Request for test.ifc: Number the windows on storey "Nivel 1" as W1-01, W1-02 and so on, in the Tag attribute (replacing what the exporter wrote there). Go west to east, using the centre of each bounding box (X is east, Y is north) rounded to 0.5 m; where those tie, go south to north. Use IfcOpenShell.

First a look at what the model holds.

```python
import ifcopenshell
import ifcopenshell.util.element
import ifcopenshell.util.placement

model = ifcopenshell.open("test.ifc")
print(model.schema)
storey = next(s for s in model.by_type("IfcBuildingStorey") if s.Name == "Nivel 1")
windows = [e for e in ifcopenshell.util.element.get_decomposition(storey) if e.is_a("IfcWindow")]
for e in sorted(windows, key=lambda e: e.id()):
    origin = ifcopenshell.util.placement.get_local_placement(e.ObjectPlacement)[:3, 3]
    print(e.id(), e.Tag, e.Name, origin.round(2) + 0.0, sep=" | ")
```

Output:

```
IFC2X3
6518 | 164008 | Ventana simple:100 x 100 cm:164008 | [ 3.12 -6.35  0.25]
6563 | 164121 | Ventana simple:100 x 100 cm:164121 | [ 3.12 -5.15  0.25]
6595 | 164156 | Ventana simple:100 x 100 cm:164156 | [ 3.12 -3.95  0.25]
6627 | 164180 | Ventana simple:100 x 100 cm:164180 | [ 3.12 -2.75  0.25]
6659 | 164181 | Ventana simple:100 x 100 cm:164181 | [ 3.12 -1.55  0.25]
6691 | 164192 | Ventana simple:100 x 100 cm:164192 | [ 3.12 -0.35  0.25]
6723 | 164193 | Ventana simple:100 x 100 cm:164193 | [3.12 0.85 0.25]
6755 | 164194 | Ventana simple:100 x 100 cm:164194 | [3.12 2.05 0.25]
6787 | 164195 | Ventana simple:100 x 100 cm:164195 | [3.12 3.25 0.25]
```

```python
import ifcopenshell
import ifcopenshell.geom
import ifcopenshell.util.element
import ifcopenshell.util.shape

model = ifcopenshell.open("test.ifc")
settings = ifcopenshell.geom.settings()
settings.set("use-world-coords", True)


def centre(element):
    shape = ifcopenshell.geom.create_shape(settings, element)
    return ifcopenshell.util.shape.get_bbox_centroid(shape.geometry)


storey = next(s for s in model.by_type("IfcBuildingStorey") if s.Name == "Nivel 1")
windows = [e for e in ifcopenshell.util.element.get_decomposition(storey) if e.is_a("IfcWindow")]

# Insertion points can sit at a corner or the storey origin, so sort by the geometry (in metres).
centres = {e: centre(e) for e in windows}
windows.sort(key=lambda e: (round(centres[e][0] / 0.5), centres[e][1]))

for i, e in enumerate(windows, start=1):
    number = f"W1-{i:02d}"
    e.Tag = number
    print(e.id(), number)

model.write("test_v2.ifc")
```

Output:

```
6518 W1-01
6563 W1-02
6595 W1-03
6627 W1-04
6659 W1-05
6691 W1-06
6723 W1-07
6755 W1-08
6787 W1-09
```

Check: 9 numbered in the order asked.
